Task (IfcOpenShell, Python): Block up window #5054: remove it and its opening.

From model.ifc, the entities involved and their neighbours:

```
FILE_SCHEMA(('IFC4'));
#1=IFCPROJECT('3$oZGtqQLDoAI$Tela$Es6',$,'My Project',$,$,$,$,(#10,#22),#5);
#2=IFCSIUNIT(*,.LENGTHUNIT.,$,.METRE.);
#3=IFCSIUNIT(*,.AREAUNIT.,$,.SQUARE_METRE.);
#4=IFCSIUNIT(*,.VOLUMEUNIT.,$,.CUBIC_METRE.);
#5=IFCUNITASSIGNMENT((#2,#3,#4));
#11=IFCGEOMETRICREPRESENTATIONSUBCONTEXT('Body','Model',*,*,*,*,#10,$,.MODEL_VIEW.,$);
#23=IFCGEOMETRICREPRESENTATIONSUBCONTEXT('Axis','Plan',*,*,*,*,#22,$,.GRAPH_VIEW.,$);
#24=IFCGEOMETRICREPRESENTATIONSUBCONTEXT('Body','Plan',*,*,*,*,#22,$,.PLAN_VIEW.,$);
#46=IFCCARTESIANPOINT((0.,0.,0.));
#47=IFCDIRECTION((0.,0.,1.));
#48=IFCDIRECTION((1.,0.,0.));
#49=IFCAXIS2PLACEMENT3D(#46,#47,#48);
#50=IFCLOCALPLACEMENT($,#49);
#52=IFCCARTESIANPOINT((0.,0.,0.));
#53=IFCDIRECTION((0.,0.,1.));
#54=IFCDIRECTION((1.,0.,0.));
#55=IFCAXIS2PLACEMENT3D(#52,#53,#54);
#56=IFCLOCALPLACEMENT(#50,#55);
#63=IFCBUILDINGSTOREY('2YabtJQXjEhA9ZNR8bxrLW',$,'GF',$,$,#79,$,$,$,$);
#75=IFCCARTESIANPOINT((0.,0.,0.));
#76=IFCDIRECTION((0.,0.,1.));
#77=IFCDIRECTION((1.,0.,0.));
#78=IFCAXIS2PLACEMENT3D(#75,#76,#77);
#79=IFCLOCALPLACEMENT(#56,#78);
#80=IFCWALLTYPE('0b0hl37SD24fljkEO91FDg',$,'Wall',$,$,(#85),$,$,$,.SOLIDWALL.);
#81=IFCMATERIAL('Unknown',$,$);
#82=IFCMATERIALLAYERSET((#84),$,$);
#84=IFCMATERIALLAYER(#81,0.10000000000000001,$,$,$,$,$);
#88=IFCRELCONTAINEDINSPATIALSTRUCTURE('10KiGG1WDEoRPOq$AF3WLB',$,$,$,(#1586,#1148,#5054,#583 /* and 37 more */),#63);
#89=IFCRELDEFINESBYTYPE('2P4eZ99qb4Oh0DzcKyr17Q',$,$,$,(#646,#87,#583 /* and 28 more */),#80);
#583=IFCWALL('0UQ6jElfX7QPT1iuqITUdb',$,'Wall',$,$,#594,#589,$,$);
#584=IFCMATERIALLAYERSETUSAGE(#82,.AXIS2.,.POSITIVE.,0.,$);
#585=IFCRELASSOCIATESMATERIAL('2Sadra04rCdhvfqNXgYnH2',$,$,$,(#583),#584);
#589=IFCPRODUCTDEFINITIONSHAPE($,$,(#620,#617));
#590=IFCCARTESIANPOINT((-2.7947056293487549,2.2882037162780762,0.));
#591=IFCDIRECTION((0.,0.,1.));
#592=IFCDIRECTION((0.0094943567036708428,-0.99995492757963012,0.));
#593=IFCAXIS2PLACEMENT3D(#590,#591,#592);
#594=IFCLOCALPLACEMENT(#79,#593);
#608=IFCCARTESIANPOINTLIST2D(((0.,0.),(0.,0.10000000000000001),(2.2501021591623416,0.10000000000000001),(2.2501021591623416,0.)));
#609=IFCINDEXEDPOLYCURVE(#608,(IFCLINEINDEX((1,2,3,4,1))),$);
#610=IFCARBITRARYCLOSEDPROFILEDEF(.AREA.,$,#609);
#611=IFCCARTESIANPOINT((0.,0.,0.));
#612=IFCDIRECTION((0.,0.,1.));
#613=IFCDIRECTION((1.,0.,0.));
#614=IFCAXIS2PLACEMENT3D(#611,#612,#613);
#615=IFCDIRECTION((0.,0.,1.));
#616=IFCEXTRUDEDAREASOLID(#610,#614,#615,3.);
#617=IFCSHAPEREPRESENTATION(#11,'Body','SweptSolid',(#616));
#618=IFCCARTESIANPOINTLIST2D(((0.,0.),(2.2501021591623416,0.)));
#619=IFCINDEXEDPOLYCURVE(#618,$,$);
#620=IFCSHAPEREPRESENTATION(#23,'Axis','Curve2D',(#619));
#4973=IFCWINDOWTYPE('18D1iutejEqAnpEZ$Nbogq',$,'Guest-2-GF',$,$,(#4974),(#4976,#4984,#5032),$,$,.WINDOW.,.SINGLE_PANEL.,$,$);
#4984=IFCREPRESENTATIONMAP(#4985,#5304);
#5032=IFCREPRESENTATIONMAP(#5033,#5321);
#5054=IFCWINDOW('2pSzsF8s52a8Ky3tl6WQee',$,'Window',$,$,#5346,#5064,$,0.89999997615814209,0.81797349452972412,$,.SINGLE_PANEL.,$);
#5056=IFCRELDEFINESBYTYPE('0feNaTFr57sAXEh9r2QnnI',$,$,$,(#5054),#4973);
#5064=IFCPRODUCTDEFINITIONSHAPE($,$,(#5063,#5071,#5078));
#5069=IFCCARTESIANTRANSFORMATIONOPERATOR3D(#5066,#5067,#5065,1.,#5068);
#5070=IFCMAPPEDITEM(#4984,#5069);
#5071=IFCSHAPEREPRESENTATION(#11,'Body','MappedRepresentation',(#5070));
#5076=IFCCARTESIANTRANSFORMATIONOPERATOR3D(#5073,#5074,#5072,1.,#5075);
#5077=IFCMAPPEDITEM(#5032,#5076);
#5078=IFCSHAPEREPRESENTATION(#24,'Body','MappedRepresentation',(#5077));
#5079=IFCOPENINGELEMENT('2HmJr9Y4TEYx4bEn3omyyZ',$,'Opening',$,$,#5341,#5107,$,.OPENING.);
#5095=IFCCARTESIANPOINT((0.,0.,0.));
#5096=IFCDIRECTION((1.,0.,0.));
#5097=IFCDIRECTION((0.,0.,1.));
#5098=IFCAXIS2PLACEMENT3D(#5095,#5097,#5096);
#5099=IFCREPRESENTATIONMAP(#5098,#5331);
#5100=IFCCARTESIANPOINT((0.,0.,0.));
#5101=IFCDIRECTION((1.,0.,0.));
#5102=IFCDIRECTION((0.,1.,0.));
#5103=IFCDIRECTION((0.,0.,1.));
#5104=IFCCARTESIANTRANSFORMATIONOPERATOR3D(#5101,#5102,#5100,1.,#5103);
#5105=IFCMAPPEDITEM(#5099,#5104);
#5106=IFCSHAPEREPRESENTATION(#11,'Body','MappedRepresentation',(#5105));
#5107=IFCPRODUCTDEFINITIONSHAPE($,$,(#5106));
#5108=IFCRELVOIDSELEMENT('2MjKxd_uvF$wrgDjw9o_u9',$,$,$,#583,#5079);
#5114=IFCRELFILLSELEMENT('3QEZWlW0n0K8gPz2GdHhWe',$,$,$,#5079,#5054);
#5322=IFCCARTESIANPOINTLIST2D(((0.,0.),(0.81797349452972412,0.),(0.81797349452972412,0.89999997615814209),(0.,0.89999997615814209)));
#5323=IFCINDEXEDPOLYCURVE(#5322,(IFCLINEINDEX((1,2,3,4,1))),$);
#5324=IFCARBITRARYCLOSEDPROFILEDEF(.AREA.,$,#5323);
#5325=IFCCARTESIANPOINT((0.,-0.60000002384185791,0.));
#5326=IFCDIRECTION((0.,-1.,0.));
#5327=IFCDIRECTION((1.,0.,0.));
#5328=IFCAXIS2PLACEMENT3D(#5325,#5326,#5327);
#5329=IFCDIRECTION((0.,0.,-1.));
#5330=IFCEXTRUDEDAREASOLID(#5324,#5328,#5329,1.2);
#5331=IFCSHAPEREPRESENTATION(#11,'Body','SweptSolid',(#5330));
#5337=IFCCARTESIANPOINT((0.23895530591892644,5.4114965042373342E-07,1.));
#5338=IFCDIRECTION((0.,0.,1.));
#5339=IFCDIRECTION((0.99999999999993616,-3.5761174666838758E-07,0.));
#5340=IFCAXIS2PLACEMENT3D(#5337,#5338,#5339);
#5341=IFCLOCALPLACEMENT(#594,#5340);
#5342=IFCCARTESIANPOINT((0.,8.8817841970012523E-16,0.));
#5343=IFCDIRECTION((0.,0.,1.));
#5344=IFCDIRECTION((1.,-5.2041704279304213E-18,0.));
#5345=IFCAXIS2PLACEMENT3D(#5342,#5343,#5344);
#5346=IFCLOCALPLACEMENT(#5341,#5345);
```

```python
import ifcopenshell
import ifcopenshell.api.feature
import ifcopenshell.api.root
import ifcopenshell.geom
import ifcopenshell.util.shape

model = ifcopenshell.open("model.ifc")
settings = ifcopenshell.geom.settings()


def volume(element):
    """Net volume in cubic metres, openings subtracted."""
    shape = ifcopenshell.geom.create_shape(settings, element)
    return ifcopenshell.util.shape.get_volume(shape.geometry)


window = model.by_guid("2pSzsF8s52a8Ky3tl6WQee")
opening = window.FillsVoids[0].RelatingOpeningElement
wall = opening.VoidsElements[0].RelatingBuildingElement
before = volume(wall)

ifcopenshell.api.root.remove_product(model, product=window)
ifcopenshell.api.feature.remove_feature(model, feature=opening)

after = volume(wall)

print(f"wall volume {before:.3f} -> {after:.3f} m3")

model.write("model-out.ifc")
```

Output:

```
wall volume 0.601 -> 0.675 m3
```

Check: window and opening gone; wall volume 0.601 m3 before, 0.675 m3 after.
